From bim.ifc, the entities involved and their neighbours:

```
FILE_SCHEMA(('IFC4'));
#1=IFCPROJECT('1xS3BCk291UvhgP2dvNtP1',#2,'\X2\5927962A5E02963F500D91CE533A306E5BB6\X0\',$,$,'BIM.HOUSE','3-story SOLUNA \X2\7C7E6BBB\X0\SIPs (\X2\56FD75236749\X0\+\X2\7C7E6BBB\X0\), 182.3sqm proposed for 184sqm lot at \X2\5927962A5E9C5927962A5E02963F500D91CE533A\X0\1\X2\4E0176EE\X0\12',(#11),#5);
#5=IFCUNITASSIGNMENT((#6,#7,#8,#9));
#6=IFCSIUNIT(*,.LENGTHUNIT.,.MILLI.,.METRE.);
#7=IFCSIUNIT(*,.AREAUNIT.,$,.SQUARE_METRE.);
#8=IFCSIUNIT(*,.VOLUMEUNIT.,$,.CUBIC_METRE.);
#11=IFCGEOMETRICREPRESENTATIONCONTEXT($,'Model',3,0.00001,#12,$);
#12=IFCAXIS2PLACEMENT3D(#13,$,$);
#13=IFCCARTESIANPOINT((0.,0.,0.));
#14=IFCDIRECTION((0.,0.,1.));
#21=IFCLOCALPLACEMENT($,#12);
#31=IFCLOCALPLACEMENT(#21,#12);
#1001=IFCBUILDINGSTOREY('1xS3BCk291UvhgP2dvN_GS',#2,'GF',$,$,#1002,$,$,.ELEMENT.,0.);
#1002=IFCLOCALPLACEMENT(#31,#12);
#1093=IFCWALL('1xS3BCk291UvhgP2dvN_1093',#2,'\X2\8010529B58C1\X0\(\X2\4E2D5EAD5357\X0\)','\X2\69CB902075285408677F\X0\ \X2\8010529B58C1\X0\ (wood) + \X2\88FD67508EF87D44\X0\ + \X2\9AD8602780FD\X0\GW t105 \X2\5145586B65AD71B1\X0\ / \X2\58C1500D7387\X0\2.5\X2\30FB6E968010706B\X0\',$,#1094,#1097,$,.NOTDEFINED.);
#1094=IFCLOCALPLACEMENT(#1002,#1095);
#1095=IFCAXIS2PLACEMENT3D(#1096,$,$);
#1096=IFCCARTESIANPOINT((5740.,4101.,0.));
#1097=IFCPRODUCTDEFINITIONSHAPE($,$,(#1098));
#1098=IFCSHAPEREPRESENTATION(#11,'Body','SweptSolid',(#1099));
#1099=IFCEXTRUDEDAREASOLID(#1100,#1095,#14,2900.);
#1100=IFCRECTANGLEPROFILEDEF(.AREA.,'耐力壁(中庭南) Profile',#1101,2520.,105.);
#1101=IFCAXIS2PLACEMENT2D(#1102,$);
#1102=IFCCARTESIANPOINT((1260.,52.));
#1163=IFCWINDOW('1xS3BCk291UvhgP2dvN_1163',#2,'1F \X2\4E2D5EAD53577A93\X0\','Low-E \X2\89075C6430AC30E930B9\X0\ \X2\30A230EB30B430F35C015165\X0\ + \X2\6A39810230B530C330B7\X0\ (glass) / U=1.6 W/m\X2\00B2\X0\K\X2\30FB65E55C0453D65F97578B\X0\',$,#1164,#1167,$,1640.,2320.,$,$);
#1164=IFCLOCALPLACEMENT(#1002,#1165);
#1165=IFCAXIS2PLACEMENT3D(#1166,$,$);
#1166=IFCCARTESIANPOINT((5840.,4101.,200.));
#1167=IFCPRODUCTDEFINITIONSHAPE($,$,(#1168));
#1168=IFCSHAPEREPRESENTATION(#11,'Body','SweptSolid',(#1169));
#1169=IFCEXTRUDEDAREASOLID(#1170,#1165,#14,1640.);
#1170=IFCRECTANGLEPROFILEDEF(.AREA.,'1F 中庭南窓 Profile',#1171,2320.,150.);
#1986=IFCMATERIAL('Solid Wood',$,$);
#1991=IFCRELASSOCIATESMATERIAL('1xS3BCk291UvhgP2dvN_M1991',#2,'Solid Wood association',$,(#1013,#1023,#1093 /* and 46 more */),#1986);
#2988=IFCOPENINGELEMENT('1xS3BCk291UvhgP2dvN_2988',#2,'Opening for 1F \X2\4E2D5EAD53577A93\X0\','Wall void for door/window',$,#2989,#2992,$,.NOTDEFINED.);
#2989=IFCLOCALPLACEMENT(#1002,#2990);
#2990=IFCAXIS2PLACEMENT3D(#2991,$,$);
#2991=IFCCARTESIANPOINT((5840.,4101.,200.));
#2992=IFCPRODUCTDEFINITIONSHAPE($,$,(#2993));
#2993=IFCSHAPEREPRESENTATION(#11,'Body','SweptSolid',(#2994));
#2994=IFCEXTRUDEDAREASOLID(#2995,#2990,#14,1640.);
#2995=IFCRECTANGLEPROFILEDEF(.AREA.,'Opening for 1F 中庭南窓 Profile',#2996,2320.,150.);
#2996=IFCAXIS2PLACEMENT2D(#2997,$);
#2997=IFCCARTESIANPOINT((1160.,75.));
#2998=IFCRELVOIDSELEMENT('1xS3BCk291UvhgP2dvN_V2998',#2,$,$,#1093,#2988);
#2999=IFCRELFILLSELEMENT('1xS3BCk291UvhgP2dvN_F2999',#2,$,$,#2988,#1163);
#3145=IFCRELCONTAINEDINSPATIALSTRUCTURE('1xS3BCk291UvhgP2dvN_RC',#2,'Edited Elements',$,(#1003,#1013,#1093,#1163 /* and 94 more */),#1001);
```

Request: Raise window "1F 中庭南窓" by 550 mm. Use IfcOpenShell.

```python
import numpy as np
import ifcopenshell
import ifcopenshell.api.geometry
import ifcopenshell.util.placement
import ifcopenshell.util.unit

model = ifcopenshell.open("bim.ifc")
unit_scale = ifcopenshell.util.unit.calculate_unit_scale(model)

window = model.by_id(1163)
opening = window.FillsVoids[0].RelatingOpeningElement
dz = 0.55 / unit_scale

shift = np.array([0.0, 0.0, dz])
# The window is not placed relative to its opening, so move both.
for product in (opening, window):
    matrix = ifcopenshell.util.placement.get_local_placement(product.ObjectPlacement)
    matrix[:3, 3] += shift
    ifcopenshell.api.geometry.edit_object_placement(model, product=product, matrix=matrix, is_si=False)

print(f"moved by {dz * unit_scale:+.3f} m")

model.write("bim-out.ifc")
```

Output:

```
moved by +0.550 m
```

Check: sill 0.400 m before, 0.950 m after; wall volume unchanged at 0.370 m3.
